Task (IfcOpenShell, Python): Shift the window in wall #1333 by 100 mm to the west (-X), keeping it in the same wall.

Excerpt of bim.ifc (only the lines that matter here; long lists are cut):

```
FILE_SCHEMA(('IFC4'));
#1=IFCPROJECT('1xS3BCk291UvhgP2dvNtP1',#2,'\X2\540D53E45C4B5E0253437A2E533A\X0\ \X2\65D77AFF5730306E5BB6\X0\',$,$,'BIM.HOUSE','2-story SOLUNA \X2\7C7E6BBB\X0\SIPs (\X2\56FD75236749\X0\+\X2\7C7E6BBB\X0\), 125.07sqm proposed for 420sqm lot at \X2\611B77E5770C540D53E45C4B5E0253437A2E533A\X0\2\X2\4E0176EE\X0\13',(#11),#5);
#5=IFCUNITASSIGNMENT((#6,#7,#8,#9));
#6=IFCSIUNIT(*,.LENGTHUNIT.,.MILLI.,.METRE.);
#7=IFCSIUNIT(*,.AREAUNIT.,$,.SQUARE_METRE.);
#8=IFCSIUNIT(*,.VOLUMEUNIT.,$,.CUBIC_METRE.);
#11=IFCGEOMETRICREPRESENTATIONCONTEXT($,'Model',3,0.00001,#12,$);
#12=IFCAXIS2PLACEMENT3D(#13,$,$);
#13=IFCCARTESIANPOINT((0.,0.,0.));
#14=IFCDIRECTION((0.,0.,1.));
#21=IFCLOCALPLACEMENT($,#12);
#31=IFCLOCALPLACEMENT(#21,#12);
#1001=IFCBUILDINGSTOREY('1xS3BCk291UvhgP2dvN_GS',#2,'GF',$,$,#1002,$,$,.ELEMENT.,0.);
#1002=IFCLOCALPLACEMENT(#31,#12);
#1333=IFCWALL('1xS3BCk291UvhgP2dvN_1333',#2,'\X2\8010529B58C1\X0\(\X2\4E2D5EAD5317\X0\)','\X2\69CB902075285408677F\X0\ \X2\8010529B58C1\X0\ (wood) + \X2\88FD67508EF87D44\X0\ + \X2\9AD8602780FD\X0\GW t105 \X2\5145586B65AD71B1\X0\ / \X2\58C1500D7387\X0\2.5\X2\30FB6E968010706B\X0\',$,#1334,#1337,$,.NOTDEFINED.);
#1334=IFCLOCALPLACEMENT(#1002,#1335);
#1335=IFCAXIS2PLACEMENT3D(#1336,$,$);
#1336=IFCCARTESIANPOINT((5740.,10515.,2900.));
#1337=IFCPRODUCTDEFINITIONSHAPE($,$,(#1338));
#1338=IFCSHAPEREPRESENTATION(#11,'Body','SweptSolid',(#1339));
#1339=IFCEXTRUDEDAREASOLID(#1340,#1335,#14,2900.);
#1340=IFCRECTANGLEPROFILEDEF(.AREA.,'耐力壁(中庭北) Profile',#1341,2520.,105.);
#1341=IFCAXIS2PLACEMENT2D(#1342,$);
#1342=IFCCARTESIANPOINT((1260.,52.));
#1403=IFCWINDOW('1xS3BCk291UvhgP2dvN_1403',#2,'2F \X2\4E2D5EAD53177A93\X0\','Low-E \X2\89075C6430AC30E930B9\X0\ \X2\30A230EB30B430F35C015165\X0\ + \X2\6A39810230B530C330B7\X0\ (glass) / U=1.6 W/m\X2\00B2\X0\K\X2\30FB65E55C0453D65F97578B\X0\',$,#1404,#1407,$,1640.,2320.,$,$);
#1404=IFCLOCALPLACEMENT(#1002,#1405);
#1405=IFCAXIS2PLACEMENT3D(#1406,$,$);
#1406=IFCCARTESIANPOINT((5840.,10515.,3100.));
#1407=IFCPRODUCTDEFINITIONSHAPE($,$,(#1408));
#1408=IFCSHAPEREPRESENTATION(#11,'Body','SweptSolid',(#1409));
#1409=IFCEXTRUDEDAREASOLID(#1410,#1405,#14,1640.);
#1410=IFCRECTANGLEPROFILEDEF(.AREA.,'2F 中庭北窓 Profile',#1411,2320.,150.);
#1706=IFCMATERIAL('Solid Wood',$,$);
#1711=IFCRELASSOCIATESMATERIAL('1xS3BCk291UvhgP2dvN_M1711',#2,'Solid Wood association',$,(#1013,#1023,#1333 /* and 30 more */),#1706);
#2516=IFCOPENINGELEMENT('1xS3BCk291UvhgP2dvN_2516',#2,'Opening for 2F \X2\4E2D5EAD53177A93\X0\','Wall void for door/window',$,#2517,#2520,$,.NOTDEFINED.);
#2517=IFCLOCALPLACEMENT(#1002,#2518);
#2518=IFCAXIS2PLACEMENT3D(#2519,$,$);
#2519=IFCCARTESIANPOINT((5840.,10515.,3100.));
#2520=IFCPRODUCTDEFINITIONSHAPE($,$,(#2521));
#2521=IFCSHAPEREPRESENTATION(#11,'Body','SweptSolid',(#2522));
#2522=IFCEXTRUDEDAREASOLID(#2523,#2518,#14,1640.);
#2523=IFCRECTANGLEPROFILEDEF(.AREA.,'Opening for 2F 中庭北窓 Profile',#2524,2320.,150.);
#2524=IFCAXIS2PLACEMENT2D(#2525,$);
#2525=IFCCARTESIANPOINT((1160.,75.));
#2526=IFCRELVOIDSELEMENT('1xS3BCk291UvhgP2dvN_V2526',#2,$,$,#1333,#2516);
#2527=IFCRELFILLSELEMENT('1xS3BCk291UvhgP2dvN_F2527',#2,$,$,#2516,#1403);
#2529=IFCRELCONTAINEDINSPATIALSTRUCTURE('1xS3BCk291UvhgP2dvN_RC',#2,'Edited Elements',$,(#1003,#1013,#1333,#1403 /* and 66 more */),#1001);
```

```python
import ifcopenshell
import ifcopenshell.api.geometry
import ifcopenshell.util.placement
import ifcopenshell.util.unit

model = ifcopenshell.open("bim.ifc")
unit_scale = ifcopenshell.util.unit.calculate_unit_scale(model)

window = model.by_guid("1xS3BCk291UvhgP2dvN_1403")
opening = window.FillsVoids[0].RelatingOpeningElement
wall = opening.VoidsElements[0].RelatingBuildingElement

wall_matrix = ifcopenshell.util.placement.get_local_placement(wall.ObjectPlacement)
shift = wall_matrix[:3, 0] * -0.1 / unit_scale
before = ifcopenshell.util.placement.get_local_placement(window.ObjectPlacement)[:3, 3].copy()

# The window is not placed relative to its opening, so move both.
for product in (opening, window):
    matrix = ifcopenshell.util.placement.get_local_placement(product.ObjectPlacement)
    matrix[:3, 3] += shift
    ifcopenshell.api.geometry.edit_object_placement(model, product=product, matrix=matrix, is_si=False)

after = ifcopenshell.util.placement.get_local_placement(window.ObjectPlacement)[:3, 3]
print("window moved by", (after - before).round(3) + 0.0)

model.write("bim_v2.ifc")
```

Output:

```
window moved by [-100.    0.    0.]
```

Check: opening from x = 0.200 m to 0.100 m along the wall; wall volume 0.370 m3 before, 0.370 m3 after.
